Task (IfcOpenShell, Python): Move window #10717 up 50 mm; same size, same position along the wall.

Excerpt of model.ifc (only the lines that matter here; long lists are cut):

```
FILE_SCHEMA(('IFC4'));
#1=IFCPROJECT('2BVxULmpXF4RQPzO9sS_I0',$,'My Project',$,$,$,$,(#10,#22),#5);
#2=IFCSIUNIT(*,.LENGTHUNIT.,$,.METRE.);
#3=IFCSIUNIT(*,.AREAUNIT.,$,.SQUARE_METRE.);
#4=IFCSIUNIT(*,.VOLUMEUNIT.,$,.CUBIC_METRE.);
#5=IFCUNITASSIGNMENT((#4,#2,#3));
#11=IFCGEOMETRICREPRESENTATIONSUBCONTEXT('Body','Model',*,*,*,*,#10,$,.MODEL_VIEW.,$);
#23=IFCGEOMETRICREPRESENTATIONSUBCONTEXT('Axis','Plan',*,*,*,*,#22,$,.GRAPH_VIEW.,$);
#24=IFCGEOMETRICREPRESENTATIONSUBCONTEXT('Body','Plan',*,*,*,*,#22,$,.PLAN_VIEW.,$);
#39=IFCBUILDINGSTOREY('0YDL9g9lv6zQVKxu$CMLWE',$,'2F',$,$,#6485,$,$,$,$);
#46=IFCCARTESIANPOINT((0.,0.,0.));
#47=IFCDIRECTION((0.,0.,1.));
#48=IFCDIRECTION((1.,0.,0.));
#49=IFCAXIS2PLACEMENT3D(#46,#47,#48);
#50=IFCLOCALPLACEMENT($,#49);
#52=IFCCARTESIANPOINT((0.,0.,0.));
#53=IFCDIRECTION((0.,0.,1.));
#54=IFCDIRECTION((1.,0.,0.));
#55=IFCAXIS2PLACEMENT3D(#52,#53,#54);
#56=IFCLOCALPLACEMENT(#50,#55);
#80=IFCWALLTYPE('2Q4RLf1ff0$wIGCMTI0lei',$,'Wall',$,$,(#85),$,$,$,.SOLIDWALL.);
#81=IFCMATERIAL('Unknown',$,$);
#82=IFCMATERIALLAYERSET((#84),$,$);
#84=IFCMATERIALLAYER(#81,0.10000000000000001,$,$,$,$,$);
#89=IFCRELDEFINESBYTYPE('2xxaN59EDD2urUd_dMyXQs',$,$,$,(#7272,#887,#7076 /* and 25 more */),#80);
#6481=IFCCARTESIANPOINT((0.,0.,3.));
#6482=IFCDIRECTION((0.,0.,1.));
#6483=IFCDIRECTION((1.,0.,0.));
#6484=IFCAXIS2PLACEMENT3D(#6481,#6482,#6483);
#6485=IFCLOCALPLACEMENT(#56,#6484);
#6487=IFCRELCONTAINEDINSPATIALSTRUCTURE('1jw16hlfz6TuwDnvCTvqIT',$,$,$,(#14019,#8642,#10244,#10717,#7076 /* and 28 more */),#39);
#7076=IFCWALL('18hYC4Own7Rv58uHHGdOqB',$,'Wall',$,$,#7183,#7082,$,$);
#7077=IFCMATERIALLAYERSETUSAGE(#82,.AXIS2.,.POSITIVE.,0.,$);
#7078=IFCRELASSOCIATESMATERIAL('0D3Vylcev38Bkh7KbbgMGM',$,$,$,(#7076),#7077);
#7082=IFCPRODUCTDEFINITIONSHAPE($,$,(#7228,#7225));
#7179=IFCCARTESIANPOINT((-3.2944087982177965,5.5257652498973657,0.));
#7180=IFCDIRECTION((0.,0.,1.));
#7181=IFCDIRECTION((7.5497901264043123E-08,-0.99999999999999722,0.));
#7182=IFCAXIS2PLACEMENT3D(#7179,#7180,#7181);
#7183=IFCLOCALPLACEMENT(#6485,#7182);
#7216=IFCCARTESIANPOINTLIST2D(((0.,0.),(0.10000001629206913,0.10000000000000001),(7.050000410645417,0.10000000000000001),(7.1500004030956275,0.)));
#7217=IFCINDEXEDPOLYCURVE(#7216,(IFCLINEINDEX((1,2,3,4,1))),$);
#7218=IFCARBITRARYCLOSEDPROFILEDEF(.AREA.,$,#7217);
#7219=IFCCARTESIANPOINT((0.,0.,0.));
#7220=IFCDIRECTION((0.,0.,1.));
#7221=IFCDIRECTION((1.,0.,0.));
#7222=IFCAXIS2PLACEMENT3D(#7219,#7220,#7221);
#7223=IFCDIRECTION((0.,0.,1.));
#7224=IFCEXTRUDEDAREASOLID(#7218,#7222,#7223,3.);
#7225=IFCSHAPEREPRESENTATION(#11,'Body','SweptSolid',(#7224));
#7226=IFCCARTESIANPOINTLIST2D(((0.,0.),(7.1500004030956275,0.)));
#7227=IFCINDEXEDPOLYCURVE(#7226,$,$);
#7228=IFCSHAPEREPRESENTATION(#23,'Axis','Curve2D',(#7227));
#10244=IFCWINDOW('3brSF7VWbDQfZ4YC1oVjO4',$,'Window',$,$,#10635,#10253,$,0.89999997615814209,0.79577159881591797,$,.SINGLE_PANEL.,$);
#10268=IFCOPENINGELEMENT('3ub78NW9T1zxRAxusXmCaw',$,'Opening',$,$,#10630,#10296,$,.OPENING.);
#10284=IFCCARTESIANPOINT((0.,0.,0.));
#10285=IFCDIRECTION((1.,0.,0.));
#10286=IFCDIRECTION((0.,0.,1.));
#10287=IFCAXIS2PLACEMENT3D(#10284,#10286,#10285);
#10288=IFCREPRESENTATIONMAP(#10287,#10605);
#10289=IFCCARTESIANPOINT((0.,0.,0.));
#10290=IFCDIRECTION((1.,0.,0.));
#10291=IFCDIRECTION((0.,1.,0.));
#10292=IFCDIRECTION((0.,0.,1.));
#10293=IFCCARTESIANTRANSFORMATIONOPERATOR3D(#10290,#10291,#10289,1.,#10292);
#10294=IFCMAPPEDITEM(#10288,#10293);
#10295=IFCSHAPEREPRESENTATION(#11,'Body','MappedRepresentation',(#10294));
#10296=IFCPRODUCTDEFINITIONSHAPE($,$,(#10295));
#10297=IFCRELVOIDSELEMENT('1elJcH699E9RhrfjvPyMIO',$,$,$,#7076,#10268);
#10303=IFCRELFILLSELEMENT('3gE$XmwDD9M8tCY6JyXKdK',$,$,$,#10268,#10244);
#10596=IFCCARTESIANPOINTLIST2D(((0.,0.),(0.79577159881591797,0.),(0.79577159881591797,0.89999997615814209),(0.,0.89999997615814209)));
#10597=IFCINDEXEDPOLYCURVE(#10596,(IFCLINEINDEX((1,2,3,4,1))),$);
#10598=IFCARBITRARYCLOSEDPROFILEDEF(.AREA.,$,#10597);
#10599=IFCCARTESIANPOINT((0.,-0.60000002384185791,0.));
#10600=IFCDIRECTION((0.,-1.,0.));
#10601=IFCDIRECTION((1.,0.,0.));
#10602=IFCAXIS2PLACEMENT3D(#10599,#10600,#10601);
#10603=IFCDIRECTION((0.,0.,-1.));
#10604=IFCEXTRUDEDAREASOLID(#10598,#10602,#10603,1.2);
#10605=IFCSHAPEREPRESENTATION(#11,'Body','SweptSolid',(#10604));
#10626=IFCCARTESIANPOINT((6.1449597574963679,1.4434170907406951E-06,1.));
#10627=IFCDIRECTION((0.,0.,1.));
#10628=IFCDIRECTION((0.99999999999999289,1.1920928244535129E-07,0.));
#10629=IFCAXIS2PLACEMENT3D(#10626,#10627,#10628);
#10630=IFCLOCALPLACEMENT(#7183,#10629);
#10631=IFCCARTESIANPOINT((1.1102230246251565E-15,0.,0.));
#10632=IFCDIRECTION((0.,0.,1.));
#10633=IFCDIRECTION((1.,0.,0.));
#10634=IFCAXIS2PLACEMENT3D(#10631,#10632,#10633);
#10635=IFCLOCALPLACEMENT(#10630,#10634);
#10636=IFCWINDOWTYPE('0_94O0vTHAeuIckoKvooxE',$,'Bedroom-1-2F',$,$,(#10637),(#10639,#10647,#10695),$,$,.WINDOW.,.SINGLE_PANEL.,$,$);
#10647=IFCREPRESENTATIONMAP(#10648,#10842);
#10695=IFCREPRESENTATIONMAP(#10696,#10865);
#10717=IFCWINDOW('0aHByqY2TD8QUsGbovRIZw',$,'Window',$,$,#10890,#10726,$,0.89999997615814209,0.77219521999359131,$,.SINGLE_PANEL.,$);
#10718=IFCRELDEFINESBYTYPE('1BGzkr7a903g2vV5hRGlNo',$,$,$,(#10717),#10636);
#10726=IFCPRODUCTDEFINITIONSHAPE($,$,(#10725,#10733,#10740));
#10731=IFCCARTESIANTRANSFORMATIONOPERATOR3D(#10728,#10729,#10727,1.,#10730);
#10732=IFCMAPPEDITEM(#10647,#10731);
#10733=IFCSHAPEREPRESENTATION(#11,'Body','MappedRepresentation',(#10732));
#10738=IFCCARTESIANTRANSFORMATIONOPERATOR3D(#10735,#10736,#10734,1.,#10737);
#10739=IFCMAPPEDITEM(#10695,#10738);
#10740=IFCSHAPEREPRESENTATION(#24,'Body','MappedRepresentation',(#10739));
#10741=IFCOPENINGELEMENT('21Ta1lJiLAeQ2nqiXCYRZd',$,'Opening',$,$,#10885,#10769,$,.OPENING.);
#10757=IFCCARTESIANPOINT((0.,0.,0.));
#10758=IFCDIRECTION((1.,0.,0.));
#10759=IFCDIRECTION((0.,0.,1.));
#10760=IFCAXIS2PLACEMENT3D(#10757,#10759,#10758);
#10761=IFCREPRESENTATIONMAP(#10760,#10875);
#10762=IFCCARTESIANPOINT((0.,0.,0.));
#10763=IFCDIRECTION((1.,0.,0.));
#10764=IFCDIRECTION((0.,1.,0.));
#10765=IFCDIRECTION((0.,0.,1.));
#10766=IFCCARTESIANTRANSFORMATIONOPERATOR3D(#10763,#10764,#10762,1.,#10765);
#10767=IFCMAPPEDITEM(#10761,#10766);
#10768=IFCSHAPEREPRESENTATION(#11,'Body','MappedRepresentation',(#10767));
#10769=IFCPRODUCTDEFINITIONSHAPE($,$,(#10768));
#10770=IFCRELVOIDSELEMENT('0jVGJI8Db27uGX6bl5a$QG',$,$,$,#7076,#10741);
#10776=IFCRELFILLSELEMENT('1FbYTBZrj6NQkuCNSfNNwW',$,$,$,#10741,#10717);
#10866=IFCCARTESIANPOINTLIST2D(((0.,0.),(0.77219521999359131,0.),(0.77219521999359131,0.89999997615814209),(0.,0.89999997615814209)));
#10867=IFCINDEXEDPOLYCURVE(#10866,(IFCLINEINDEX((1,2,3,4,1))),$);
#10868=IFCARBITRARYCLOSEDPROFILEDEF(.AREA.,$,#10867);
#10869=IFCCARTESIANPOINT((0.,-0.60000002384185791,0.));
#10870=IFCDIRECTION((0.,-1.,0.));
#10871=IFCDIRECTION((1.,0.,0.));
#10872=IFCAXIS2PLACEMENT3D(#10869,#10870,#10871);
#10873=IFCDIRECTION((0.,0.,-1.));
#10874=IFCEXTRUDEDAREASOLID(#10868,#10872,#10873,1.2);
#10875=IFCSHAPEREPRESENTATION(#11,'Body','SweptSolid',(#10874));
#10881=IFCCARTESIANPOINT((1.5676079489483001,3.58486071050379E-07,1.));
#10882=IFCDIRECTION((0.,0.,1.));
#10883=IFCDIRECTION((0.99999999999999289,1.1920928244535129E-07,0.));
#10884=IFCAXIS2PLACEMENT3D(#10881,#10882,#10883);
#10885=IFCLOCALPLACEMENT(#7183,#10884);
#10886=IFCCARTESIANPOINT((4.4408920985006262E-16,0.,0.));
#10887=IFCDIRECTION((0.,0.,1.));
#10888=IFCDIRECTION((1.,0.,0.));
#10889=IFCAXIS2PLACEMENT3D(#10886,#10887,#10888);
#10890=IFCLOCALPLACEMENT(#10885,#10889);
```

```python
import numpy as np
import ifcopenshell
import ifcopenshell.api.geometry
import ifcopenshell.util.placement
import ifcopenshell.util.unit

model = ifcopenshell.open("model.ifc")
unit_scale = ifcopenshell.util.unit.calculate_unit_scale(model)

window = model.by_id(10717)
opening = window.FillsVoids[0].RelatingOpeningElement
dz = 0.05

shift = np.array([0.0, 0.0, dz])
# The window is placed relative to its opening, so it follows when the opening moves.
matrix = ifcopenshell.util.placement.get_local_placement(opening.ObjectPlacement)
matrix[:3, 3] += shift
ifcopenshell.api.geometry.edit_object_placement(
    model, product=opening, matrix=matrix, is_si=False, should_transform_children=True
)

print(f"moved by {dz * unit_scale:+.3f} m")

model.write("model_v2.ifc")
```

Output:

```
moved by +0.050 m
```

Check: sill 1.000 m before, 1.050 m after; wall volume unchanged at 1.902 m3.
